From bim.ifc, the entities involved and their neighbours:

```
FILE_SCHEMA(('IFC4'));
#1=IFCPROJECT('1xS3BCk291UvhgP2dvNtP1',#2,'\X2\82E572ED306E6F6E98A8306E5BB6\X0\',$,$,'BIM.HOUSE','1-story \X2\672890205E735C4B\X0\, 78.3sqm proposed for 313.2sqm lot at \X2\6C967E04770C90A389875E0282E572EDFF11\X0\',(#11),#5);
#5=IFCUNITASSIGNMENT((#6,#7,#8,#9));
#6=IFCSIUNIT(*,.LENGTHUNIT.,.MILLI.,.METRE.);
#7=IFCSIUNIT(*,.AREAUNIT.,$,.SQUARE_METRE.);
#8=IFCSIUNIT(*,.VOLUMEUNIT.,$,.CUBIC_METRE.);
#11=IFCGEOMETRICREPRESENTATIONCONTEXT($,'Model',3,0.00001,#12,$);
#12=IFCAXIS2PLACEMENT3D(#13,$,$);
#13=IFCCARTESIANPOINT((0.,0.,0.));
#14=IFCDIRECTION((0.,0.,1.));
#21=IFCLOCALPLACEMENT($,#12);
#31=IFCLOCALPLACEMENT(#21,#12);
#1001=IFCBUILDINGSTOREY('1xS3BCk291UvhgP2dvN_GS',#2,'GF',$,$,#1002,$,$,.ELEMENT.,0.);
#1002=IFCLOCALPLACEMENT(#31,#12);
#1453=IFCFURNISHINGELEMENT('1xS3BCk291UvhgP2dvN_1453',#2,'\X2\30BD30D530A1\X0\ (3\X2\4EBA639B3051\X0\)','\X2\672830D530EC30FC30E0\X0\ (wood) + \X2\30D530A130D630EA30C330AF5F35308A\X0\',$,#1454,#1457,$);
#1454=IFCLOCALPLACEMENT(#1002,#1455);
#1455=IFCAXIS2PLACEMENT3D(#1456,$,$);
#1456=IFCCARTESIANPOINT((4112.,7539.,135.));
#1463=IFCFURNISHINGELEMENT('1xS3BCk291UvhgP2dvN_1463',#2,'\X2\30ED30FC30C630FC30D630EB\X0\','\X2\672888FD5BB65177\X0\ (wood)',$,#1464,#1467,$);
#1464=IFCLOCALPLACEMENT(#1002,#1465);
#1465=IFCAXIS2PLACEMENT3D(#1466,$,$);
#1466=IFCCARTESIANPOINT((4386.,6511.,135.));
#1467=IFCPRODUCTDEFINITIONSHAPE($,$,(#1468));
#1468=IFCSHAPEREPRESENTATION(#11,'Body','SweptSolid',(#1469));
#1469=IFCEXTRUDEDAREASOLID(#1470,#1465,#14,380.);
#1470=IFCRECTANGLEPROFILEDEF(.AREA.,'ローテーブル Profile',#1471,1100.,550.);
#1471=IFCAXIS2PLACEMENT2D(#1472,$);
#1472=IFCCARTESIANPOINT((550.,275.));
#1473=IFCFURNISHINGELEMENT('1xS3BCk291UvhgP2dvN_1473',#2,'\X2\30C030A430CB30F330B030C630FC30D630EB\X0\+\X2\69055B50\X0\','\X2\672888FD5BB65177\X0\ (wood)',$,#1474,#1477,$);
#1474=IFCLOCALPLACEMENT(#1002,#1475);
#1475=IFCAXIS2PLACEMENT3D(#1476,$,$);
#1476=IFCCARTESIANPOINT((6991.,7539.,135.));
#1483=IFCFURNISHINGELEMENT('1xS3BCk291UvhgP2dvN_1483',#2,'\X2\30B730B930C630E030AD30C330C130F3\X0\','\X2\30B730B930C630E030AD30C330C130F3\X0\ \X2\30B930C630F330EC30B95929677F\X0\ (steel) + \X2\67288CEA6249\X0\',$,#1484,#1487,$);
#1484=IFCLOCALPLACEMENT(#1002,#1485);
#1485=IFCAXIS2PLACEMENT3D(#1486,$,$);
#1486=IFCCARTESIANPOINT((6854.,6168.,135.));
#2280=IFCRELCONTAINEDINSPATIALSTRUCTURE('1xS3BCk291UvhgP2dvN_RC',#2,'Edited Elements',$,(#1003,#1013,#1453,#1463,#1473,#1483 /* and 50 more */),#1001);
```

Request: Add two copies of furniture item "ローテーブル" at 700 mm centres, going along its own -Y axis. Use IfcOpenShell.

```python
import ifcopenshell
import ifcopenshell.api.geometry
import ifcopenshell.api.root
import ifcopenshell.util.element
import ifcopenshell.util.placement
import ifcopenshell.util.unit

model = ifcopenshell.open("bim.ifc")
unit_scale = ifcopenshell.util.unit.calculate_unit_scale(model)


def reuse_history(source, copy):
    """copy_class also copies each property set's owner history, people and application; keep the originals."""
    for rel in copy.IsDefinedBy:
        if rel.is_a("IfcRelDefinesByProperties") and (history := rel.RelatingPropertyDefinition.OwnerHistory):
            rel.RelatingPropertyDefinition.OwnerHistory = source.OwnerHistory
            ifcopenshell.util.element.remove_deep2(model, history)


source = model.by_id(1463)
base = ifcopenshell.util.placement.get_local_placement(source.ObjectPlacement)
step = -base[:3, 1] * 0.7 / unit_scale

for i in range(1, 3):
    copy = ifcopenshell.api.root.copy_class(model, product=source)
    copy.Representation = ifcopenshell.util.element.copy_deep(
        model, source.Representation, exclude=["IfcGeometricRepresentationContext", "IfcRepresentationMap"]
    )
    reuse_history(source, copy)
    matrix = base.copy()
    matrix[:3, 3] += i * step
    print("added at", matrix[:3, 3].round(3) + 0.0)
    ifcopenshell.api.geometry.edit_object_placement(model, product=copy, matrix=matrix, is_si=False)

model.write("bim_v2.ifc")
```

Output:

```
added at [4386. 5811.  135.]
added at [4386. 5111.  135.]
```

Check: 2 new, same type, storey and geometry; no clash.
